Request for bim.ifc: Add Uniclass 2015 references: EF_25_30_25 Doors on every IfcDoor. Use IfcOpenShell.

First a look at what the model holds.

```python
import ifcopenshell

model = ifcopenshell.open("bim.ifc")
print(model.schema)
print("classifications:", [c.Name for c in model.by_type("IfcClassification")])
for ifc_class in ("IfcDoor", "IfcRoof", "IfcStair", "IfcWall", "IfcWindow"):
    print(ifc_class, len(model.by_type(ifc_class)))
```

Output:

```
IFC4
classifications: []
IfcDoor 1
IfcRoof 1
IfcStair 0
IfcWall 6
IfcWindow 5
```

```python
import ifcopenshell
import ifcopenshell.api.classification

model = ifcopenshell.open("bim.ifc")

system = ifcopenshell.api.classification.add_classification(model, classification="Uniclass 2015")

codes = {
    "IfcDoor": ("EF_25_30_25", "Doors"),
}
for ifc_class, (code, name) in codes.items():
    products = model.by_type(ifc_class)
    ifcopenshell.api.classification.add_reference(
        model, products=products, classification=system, identification=code, name=name
    )
    print(code, len(products))

model.write("bim_edited.ifc")
```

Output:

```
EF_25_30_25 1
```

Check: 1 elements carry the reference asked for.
